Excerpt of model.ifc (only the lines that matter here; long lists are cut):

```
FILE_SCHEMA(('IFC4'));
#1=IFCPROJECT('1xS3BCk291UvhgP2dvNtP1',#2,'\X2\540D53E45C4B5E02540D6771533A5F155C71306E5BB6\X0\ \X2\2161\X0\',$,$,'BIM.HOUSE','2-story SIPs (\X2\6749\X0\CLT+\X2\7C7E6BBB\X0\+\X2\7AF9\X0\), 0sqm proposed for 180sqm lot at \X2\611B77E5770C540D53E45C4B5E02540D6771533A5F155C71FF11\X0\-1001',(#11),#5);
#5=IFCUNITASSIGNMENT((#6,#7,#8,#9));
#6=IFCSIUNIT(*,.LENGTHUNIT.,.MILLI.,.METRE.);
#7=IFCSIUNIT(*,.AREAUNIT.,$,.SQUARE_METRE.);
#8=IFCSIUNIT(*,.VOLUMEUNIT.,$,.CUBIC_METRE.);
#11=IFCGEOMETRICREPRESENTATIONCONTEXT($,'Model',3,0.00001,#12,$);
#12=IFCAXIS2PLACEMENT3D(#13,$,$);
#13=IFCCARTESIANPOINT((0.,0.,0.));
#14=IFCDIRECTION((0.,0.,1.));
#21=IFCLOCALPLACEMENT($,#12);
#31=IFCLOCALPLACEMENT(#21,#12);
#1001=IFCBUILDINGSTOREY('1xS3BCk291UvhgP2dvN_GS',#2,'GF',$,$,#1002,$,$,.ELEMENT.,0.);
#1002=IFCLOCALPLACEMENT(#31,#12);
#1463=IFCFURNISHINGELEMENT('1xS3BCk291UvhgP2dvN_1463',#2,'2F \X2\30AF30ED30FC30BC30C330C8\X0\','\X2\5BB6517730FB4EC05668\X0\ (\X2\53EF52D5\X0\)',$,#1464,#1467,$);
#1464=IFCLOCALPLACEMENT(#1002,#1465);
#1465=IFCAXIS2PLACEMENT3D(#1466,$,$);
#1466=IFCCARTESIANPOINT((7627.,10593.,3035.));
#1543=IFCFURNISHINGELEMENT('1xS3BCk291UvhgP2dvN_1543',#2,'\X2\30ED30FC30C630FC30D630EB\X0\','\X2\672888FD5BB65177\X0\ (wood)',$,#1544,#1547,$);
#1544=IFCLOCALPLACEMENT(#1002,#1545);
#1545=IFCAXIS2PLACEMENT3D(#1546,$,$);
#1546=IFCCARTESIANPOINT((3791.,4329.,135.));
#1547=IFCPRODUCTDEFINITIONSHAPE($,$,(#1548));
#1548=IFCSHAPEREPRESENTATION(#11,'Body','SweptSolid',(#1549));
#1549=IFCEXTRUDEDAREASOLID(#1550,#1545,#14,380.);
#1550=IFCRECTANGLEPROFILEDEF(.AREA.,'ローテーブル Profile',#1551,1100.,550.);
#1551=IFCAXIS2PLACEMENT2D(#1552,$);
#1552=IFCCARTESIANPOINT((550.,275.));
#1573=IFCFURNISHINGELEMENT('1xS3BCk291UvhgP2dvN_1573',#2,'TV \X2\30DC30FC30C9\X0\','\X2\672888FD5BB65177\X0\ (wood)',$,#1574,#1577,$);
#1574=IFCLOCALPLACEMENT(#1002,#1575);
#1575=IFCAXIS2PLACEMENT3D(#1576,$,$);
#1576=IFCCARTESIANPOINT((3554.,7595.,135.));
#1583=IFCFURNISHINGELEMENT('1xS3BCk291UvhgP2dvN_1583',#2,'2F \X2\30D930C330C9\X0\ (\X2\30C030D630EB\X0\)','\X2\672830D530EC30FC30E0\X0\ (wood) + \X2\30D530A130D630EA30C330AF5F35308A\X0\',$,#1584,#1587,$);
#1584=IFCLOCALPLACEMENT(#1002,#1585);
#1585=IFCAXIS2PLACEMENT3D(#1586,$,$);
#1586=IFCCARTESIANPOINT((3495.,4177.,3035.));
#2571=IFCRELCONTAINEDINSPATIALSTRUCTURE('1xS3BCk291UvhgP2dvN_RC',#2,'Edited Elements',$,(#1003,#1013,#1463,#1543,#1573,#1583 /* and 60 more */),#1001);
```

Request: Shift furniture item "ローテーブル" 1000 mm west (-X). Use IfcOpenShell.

```python
import ifcopenshell
import ifcopenshell.api.geometry
import ifcopenshell.util.placement
import ifcopenshell.util.unit

model = ifcopenshell.open("model.ifc")
unit_scale = ifcopenshell.util.unit.calculate_unit_scale(model)

item = model.by_guid("1xS3BCk291UvhgP2dvN_1543")
matrix = ifcopenshell.util.placement.get_local_placement(item.ObjectPlacement)
matrix[0, 3] -= 1 / unit_scale
ifcopenshell.api.geometry.edit_object_placement(model, product=item, matrix=matrix, is_si=False)

print(ifcopenshell.util.placement.get_local_placement(item.ObjectPlacement).round(3) + 0.0)

model.write("model_rev.ifc")
```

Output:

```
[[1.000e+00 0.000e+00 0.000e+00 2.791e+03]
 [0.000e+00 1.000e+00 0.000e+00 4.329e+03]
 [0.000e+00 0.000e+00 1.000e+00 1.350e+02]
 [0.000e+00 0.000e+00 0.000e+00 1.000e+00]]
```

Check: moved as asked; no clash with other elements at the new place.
